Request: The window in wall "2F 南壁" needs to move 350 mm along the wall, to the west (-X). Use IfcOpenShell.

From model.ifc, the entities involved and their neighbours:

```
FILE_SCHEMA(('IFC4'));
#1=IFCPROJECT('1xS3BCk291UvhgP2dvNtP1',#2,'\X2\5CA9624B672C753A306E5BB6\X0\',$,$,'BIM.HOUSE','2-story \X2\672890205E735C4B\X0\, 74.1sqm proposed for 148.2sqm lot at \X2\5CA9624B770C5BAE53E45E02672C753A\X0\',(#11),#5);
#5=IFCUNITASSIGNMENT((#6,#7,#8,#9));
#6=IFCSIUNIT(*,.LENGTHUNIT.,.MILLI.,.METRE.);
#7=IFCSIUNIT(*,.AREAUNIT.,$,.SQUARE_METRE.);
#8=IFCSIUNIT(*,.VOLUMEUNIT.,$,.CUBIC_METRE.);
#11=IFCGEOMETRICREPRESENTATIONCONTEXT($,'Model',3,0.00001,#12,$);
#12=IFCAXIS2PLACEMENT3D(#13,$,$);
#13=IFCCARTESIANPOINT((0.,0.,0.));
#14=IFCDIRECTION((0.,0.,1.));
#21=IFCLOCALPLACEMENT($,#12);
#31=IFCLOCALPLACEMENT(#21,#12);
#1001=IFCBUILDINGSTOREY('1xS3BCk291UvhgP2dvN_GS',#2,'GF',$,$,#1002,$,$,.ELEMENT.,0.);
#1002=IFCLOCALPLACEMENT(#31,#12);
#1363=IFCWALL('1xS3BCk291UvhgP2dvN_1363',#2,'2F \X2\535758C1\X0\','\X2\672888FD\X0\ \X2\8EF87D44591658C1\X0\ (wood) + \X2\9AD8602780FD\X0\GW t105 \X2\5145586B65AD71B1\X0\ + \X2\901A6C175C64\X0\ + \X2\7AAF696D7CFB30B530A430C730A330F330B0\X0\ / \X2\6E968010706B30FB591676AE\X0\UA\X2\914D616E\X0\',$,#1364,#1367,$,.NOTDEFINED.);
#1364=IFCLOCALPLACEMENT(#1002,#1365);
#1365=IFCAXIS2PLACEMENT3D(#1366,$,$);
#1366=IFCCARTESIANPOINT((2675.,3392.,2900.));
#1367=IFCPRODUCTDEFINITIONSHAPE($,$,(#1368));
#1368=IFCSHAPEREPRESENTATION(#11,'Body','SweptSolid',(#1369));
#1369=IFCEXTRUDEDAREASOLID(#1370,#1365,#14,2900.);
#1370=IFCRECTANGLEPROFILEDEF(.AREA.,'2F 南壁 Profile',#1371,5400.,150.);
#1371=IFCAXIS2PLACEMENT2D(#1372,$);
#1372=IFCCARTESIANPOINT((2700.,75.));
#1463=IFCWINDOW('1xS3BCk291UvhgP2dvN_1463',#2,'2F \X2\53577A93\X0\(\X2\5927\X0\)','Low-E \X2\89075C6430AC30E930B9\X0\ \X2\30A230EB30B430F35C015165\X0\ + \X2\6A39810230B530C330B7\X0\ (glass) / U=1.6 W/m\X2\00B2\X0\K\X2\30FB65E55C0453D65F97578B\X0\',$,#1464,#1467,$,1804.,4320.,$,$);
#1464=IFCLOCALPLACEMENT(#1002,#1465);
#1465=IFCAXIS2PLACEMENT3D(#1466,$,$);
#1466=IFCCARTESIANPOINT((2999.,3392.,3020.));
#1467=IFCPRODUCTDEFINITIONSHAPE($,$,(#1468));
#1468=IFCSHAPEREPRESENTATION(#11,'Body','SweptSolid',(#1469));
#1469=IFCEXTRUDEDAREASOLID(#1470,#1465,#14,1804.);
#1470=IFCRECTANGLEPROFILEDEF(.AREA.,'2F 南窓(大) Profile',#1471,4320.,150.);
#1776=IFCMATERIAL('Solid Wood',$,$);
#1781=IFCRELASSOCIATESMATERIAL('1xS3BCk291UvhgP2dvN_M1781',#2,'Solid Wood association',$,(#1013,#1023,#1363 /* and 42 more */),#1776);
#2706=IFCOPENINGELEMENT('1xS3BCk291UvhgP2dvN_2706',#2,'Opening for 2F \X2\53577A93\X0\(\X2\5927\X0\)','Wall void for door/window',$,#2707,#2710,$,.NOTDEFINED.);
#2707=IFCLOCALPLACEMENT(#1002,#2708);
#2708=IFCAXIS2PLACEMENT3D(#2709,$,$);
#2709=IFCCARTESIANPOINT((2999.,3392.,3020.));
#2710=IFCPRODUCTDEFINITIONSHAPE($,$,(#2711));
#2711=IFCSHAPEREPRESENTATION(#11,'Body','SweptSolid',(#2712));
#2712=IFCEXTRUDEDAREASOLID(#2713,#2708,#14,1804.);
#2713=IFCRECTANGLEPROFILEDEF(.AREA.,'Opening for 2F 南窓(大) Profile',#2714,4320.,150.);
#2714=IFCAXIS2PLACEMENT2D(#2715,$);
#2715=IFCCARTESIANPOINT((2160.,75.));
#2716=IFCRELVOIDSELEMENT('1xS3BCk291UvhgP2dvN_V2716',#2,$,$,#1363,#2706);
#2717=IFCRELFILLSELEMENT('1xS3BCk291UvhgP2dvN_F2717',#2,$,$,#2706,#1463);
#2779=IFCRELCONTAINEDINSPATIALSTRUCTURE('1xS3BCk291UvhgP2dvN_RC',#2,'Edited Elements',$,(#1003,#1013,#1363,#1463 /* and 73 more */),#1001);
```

```python
import ifcopenshell
import ifcopenshell.api.geometry
import ifcopenshell.util.placement
import ifcopenshell.util.unit

model = ifcopenshell.open("model.ifc")
unit_scale = ifcopenshell.util.unit.calculate_unit_scale(model)

window = model.by_guid("1xS3BCk291UvhgP2dvN_1463")
opening = window.FillsVoids[0].RelatingOpeningElement
wall = opening.VoidsElements[0].RelatingBuildingElement

wall_matrix = ifcopenshell.util.placement.get_local_placement(wall.ObjectPlacement)
shift = wall_matrix[:3, 0] * -0.35 / unit_scale
before = ifcopenshell.util.placement.get_local_placement(window.ObjectPlacement)[:3, 3].copy()

# The window is not placed relative to its opening, so move both.
for product in (opening, window):
    matrix = ifcopenshell.util.placement.get_local_placement(product.ObjectPlacement)
    matrix[:3, 3] += shift
    ifcopenshell.api.geometry.edit_object_placement(model, product=product, matrix=matrix, is_si=False)

after = ifcopenshell.util.placement.get_local_placement(window.ObjectPlacement)[:3, 3]
print("window moved by", (after - before).round(3) + 0.0)

model.write("model-out.ifc")
```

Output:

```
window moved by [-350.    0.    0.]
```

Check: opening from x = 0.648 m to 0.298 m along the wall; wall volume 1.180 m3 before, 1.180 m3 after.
